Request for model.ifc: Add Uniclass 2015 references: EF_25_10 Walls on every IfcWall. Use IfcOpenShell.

First a look at what the model holds.

```python
import ifcopenshell

model = ifcopenshell.open("model.ifc")
print(model.schema)
print("classifications:", [c.Name for c in model.by_type("IfcClassification")])
for ifc_class in ("IfcDoor", "IfcRoof", "IfcStair", "IfcWall", "IfcWindow"):
    print(ifc_class, len(model.by_type(ifc_class)))
```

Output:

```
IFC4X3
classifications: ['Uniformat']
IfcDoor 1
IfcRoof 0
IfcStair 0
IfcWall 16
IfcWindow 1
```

```python
import ifcopenshell
import ifcopenshell.api.classification

model = ifcopenshell.open("model.ifc")

system = ifcopenshell.api.classification.add_classification(model, classification="Uniclass 2015")

codes = {
    "IfcWall": ("EF_25_10", "Walls"),
}
for ifc_class, (code, name) in codes.items():
    products = model.by_type(ifc_class)
    ifcopenshell.api.classification.add_reference(
        model, products=products, classification=system, identification=code, name=name
    )
    print(code, len(products))

model.write("model_edited.ifc")
```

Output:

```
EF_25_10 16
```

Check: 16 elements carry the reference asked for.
